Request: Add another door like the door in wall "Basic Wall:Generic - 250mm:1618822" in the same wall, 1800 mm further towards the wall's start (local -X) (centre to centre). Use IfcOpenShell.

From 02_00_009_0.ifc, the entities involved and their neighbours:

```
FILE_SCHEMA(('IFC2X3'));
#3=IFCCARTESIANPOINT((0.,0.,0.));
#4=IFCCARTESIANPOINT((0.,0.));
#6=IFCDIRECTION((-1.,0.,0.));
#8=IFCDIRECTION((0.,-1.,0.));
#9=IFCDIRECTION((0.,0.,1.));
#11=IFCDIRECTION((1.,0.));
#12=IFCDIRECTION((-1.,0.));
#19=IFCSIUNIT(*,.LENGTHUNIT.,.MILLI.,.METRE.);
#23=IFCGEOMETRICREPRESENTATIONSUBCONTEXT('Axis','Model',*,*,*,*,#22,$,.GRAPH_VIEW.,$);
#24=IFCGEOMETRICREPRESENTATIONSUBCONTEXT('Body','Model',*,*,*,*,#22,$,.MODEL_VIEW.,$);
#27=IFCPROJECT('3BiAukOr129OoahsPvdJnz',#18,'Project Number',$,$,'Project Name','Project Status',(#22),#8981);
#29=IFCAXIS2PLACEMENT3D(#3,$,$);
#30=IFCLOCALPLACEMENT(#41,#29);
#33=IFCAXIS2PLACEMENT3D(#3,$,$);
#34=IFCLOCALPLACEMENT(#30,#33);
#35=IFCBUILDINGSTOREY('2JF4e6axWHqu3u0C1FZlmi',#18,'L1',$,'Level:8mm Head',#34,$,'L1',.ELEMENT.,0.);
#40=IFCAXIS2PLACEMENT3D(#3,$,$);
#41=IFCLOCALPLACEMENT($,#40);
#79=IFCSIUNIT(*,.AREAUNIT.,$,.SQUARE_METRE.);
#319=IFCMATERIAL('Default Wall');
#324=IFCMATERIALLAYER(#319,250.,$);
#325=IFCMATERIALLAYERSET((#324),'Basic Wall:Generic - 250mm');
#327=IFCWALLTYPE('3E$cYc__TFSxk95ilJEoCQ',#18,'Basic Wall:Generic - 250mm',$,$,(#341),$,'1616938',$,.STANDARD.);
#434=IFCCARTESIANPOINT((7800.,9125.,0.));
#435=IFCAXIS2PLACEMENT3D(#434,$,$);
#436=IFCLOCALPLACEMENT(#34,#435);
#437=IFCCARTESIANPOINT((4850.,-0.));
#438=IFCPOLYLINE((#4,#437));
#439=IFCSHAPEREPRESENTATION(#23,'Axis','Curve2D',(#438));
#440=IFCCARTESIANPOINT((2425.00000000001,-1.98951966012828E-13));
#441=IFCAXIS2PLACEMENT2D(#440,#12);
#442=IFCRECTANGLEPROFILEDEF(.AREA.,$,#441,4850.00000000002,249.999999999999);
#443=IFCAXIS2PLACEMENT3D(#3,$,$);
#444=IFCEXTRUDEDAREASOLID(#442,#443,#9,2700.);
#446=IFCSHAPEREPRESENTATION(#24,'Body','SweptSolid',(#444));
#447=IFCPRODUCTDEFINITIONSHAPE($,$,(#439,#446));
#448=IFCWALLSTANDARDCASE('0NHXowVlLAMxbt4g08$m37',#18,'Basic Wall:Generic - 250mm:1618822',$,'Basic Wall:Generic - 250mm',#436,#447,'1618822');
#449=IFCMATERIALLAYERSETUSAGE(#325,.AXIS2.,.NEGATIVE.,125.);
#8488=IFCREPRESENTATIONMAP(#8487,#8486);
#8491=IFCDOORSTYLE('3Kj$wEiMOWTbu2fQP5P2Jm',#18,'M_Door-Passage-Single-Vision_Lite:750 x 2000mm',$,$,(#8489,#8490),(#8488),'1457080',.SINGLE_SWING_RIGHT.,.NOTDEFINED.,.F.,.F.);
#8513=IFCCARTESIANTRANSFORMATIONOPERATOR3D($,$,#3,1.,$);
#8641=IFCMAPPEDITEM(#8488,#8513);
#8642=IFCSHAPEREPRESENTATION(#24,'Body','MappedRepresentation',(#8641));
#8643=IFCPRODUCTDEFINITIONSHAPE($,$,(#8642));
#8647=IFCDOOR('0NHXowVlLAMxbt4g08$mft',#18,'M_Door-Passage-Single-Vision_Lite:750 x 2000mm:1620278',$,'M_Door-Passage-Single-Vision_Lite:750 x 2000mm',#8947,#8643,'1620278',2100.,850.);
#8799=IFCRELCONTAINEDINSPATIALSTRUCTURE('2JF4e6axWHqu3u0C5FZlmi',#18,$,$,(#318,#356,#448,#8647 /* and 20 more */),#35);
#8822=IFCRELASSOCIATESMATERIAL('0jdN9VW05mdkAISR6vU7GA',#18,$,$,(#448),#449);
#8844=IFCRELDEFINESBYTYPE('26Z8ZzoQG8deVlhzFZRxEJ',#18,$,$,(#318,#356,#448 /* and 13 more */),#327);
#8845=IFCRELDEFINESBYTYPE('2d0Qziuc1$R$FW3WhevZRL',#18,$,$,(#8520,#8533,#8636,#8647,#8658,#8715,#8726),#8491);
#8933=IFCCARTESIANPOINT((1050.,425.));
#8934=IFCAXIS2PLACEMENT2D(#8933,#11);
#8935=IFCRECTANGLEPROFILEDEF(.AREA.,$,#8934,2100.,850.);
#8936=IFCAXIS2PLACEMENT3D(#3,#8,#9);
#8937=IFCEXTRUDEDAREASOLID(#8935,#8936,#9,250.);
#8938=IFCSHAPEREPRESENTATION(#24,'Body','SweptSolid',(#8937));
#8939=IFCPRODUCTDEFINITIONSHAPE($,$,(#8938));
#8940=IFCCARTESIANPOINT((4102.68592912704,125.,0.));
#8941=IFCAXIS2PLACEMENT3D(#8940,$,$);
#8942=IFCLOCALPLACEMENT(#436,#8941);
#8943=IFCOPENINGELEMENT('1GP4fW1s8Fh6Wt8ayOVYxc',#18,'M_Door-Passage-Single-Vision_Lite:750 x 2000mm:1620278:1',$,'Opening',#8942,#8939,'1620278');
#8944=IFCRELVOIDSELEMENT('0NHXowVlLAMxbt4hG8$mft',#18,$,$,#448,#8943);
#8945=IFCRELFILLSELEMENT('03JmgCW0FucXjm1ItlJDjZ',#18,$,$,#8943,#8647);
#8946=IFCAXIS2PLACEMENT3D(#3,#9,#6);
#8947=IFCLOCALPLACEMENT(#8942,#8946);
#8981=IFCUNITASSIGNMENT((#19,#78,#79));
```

```python
import ifcopenshell
import ifcopenshell.api.feature
import ifcopenshell.api.geometry
import ifcopenshell.api.root
import ifcopenshell.geom
import ifcopenshell.util.element
import ifcopenshell.util.placement
import ifcopenshell.util.shape

model = ifcopenshell.open("02_00_009_0.ifc")
settings = ifcopenshell.geom.settings()


def volume(element):
    """Net volume in cubic metres, openings subtracted."""
    shape = ifcopenshell.geom.create_shape(settings, element)
    return ifcopenshell.util.shape.get_volume(shape.geometry)


def reuse_history(source, copy):
    """copy_class also copies each property set's owner history, people and application; keep the originals."""
    for rel in copy.IsDefinedBy:
        if rel.is_a("IfcRelDefinesByProperties") and (history := rel.RelatingPropertyDefinition.OwnerHistory):
            rel.RelatingPropertyDefinition.OwnerHistory = source.OwnerHistory
            ifcopenshell.util.element.remove_deep2(model, history)


door = model.by_guid("0NHXowVlLAMxbt4g08$mft")
opening = door.FillsVoids[0].RelatingOpeningElement
wall = opening.VoidsElements[0].RelatingBuildingElement
before = volume(wall)
shift = ifcopenshell.util.placement.get_local_placement(wall.ObjectPlacement)[:3, 0] * -1800.0

# copy_class copies the void relationship, type, container and properties, but no geometry.
new_opening = ifcopenshell.api.root.copy_class(model, product=opening)
new_opening.Representation = ifcopenshell.util.element.copy_deep(
    model, opening.Representation, exclude=["IfcGeometricRepresentationContext", "IfcRepresentationMap"]
)
new_opening.Name = "M_Door-Passage-Single-Vision_Lite:750 x 2000mm"
new_opening.Tag = None
new_door = ifcopenshell.api.root.copy_class(model, product=door)
new_door.Representation = ifcopenshell.util.element.copy_deep(
    model, door.Representation, exclude=["IfcGeometricRepresentationContext", "IfcRepresentationMap"]
)
new_door.Name = "M_Door-Passage-Single-Vision_Lite:750 x 2000mm"
new_door.Tag = None
reuse_history(door, new_door)
fills = ifcopenshell.api.feature.add_filling(model, opening=new_opening, element=new_door)
fills.OwnerHistory = new_door.OwnerHistory  # required in IFC2X3

for old, new in ((opening, new_opening), (door, new_door)):
    matrix = ifcopenshell.util.placement.get_local_placement(old.ObjectPlacement)
    matrix[:3, 3] += shift
    ifcopenshell.api.geometry.edit_object_placement(model, product=new, matrix=matrix, is_si=False)

after = volume(wall)

print(f"wall volume {before:.3f} -> {after:.3f} m3")

model.write("02_00_009_0_updated.ifc")
```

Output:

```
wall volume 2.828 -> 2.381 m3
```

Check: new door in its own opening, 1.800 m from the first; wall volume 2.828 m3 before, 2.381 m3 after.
